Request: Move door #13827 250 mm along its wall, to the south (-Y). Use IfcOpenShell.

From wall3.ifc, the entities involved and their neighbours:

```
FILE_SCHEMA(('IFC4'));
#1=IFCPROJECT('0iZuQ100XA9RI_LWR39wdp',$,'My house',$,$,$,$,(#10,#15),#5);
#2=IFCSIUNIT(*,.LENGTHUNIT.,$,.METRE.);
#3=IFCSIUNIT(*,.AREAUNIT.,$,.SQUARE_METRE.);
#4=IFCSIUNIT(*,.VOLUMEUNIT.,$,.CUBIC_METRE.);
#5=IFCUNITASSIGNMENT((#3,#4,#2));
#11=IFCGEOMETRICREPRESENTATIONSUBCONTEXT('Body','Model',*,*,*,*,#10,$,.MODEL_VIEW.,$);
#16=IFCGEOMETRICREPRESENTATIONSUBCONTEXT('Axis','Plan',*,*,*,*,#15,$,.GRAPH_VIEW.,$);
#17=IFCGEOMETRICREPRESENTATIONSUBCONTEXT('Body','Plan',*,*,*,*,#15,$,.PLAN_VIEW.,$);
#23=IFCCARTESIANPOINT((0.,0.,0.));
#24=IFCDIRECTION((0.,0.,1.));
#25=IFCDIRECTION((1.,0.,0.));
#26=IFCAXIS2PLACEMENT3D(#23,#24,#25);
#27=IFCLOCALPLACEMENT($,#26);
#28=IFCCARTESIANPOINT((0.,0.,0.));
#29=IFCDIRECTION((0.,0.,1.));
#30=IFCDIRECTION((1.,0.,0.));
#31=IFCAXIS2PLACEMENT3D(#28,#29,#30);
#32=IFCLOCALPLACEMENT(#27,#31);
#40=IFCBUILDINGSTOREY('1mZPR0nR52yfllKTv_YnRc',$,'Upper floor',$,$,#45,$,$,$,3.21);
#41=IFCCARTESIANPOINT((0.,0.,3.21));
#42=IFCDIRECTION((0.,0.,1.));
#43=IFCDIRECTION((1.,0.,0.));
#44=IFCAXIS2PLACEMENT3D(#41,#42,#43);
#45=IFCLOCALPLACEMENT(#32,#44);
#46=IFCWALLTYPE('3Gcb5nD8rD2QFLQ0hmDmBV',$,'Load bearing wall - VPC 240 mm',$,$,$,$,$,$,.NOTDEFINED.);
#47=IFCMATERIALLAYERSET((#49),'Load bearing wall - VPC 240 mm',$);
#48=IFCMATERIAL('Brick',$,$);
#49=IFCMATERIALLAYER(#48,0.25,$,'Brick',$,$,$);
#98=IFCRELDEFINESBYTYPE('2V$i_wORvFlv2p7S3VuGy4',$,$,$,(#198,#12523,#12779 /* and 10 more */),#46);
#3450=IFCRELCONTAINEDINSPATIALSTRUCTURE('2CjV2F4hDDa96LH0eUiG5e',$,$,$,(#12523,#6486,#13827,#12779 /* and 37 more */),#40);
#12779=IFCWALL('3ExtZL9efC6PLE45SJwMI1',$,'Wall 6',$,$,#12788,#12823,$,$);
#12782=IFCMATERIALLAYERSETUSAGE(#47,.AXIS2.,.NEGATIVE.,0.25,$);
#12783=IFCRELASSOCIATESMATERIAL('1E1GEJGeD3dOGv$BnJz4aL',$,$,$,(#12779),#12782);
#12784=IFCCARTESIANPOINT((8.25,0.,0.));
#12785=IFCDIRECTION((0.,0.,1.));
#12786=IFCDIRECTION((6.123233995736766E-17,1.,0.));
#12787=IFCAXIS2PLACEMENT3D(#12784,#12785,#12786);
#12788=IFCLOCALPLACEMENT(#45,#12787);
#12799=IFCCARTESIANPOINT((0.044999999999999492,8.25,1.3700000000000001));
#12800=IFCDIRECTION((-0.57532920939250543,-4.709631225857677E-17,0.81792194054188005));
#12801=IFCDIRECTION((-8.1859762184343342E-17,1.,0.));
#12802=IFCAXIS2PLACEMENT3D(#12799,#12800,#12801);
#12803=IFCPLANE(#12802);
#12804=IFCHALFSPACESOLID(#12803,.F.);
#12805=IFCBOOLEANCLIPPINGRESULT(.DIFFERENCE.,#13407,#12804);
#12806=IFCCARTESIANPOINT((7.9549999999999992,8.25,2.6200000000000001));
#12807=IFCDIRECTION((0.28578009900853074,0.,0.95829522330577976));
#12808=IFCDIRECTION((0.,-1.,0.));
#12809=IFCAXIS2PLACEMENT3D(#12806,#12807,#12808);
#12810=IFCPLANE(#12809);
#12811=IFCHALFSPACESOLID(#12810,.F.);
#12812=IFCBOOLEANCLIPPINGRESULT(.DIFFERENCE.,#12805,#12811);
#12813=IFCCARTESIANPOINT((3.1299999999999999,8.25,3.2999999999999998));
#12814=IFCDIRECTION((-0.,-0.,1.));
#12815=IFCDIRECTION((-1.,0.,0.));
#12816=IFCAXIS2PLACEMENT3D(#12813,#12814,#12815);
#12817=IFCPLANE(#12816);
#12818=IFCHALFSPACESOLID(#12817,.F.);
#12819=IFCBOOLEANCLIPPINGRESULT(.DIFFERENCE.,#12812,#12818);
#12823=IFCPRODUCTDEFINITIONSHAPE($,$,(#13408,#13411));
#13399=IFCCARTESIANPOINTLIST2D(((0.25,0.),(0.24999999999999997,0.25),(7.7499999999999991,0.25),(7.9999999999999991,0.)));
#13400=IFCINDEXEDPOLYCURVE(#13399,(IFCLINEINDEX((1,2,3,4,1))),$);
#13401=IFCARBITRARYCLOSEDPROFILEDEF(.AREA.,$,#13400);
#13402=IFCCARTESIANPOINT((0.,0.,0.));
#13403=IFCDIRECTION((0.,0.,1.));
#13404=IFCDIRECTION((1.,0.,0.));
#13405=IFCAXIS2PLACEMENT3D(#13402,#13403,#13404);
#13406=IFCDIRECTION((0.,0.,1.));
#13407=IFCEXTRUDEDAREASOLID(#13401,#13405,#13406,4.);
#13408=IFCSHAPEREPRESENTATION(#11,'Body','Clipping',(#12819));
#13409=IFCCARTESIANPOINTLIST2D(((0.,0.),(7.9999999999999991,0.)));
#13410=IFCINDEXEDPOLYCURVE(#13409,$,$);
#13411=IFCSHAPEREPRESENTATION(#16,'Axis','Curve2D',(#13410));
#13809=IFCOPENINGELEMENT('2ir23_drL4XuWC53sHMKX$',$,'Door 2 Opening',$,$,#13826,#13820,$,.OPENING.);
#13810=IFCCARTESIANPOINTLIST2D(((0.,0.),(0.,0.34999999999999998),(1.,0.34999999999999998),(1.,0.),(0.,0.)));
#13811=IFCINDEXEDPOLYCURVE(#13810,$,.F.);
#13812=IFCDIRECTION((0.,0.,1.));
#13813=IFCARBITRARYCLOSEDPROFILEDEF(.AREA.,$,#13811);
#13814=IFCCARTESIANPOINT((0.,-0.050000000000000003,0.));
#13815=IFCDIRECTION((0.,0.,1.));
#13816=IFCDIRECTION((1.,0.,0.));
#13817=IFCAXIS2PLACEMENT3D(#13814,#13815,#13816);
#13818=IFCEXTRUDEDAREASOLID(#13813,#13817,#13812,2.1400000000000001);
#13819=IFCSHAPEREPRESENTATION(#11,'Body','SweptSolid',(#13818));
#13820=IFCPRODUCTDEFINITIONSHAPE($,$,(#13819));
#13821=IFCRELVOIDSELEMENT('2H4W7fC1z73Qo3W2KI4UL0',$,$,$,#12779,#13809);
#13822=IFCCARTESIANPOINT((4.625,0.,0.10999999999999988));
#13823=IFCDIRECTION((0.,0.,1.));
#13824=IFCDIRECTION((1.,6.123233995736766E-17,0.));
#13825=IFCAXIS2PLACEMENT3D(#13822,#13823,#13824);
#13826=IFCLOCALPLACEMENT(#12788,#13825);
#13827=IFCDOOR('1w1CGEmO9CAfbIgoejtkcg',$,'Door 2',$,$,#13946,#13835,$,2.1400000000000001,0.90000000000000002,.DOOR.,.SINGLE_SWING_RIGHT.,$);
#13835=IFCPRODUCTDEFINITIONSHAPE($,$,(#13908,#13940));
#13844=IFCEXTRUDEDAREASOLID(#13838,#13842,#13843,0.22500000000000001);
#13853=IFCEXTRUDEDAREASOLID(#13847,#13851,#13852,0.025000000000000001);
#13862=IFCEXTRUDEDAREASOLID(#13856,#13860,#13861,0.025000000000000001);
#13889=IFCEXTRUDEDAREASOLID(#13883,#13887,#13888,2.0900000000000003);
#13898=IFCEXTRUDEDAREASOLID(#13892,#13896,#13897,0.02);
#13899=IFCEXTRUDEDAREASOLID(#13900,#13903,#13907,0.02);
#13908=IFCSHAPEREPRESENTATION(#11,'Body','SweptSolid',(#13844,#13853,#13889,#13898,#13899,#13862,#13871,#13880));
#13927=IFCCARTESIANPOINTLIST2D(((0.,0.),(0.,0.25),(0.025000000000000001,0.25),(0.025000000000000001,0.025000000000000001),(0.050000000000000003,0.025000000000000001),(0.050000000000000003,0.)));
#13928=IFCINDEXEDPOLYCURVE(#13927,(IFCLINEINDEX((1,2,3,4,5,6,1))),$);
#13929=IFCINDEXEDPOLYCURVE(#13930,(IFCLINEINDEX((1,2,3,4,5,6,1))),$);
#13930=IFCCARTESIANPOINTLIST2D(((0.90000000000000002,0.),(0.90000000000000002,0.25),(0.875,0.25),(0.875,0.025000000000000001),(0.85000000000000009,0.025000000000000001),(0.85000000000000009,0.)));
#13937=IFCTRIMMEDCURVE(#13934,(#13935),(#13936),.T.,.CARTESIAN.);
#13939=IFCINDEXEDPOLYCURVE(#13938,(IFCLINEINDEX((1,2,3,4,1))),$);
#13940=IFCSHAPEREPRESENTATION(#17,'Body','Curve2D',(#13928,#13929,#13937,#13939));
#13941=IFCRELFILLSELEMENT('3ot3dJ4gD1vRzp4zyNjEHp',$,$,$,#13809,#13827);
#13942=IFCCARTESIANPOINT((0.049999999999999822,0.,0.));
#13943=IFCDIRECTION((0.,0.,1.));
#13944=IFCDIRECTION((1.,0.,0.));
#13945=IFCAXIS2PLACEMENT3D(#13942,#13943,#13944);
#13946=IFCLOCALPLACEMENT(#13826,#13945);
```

```python
import ifcopenshell
import ifcopenshell.api.geometry
import ifcopenshell.util.placement

model = ifcopenshell.open("wall3.ifc")

door = model.by_guid("1w1CGEmO9CAfbIgoejtkcg")
opening = door.FillsVoids[0].RelatingOpeningElement
wall = opening.VoidsElements[0].RelatingBuildingElement

wall_matrix = ifcopenshell.util.placement.get_local_placement(wall.ObjectPlacement)
shift = wall_matrix[:3, 0] * -0.25
before = ifcopenshell.util.placement.get_local_placement(door.ObjectPlacement)[:3, 3].copy()

# The door is placed relative to its opening, so it follows when the opening moves.
matrix = ifcopenshell.util.placement.get_local_placement(opening.ObjectPlacement)
matrix[:3, 3] += shift
ifcopenshell.api.geometry.edit_object_placement(
    model, product=opening, matrix=matrix, is_si=False, should_transform_children=True
)

after = ifcopenshell.util.placement.get_local_placement(door.ObjectPlacement)[:3, 3]
print("door moved by", (after - before).round(3) + 0.0)

model.write("wall3_edited.ifc")
```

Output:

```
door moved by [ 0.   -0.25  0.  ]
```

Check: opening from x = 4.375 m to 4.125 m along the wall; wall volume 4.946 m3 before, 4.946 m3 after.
